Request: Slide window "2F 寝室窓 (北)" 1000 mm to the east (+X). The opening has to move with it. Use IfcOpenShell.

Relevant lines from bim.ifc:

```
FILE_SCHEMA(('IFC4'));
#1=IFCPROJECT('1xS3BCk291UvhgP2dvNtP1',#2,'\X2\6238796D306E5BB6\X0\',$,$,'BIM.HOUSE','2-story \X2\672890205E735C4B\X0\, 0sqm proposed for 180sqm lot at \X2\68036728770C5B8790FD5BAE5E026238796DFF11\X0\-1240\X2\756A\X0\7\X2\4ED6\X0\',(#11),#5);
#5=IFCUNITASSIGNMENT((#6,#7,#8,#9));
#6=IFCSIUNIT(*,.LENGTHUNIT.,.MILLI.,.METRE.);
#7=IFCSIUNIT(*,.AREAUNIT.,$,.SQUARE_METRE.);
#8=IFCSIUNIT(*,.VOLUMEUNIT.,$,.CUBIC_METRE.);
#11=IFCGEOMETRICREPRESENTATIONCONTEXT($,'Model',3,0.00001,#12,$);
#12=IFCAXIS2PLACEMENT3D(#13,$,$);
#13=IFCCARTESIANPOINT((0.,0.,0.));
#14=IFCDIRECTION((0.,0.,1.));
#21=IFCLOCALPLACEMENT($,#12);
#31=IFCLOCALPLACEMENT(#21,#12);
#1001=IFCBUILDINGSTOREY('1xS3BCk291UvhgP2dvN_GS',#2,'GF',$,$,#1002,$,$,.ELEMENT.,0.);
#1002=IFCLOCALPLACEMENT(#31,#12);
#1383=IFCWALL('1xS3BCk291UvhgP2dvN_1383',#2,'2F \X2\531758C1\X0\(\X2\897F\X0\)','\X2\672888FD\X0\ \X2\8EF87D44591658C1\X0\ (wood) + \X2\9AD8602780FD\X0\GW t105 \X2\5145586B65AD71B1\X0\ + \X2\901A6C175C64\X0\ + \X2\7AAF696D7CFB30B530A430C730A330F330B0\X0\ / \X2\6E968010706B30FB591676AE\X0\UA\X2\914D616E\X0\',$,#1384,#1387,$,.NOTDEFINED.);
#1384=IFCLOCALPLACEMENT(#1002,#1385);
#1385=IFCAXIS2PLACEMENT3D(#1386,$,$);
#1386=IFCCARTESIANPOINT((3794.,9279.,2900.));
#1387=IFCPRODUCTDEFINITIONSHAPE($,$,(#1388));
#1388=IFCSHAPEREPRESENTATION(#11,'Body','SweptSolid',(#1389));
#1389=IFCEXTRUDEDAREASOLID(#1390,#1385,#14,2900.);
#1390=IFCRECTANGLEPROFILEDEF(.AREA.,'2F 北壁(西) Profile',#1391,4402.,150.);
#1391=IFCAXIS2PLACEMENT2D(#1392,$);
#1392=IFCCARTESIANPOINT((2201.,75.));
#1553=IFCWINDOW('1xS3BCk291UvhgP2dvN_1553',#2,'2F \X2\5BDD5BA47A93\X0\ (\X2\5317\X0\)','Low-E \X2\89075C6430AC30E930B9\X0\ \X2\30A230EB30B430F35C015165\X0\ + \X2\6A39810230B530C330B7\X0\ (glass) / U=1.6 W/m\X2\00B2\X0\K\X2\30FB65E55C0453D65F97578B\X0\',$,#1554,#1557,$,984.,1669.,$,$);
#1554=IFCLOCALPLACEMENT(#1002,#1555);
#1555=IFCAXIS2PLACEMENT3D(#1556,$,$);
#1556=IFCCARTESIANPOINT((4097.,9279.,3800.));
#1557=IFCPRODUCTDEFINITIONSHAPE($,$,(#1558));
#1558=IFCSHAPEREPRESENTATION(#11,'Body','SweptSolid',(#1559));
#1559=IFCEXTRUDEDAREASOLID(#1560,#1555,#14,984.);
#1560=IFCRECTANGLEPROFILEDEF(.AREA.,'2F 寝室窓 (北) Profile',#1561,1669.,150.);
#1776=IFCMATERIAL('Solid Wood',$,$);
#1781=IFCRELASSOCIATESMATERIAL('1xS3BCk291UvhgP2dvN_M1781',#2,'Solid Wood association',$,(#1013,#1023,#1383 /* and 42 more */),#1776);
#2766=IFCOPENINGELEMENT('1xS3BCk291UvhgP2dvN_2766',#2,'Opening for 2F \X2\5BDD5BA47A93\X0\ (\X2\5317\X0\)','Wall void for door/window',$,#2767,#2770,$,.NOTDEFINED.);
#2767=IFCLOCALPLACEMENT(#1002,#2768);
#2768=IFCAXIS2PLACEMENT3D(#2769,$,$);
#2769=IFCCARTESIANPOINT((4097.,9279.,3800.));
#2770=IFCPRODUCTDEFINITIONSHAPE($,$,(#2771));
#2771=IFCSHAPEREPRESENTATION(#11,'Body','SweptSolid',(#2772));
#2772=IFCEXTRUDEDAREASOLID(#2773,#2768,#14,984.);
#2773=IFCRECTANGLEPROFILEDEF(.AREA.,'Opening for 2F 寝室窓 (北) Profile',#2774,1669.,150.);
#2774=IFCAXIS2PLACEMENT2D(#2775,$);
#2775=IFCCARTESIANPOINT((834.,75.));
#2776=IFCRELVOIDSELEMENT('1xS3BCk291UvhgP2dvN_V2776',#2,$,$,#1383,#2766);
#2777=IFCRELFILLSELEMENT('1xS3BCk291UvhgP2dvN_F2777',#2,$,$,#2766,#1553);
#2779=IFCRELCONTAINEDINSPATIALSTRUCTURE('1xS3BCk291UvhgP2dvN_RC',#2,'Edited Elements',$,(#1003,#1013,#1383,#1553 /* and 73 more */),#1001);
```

```python
import ifcopenshell
import ifcopenshell.api.geometry
import ifcopenshell.util.placement
import ifcopenshell.util.unit

model = ifcopenshell.open("bim.ifc")
unit_scale = ifcopenshell.util.unit.calculate_unit_scale(model)

window = model.by_id(1553)
opening = window.FillsVoids[0].RelatingOpeningElement
wall = opening.VoidsElements[0].RelatingBuildingElement

wall_matrix = ifcopenshell.util.placement.get_local_placement(wall.ObjectPlacement)
shift = wall_matrix[:3, 0] * 1 / unit_scale
before = ifcopenshell.util.placement.get_local_placement(window.ObjectPlacement)[:3, 3].copy()

# The window is not placed relative to its opening, so move both.
for product in (opening, window):
    matrix = ifcopenshell.util.placement.get_local_placement(product.ObjectPlacement)
    matrix[:3, 3] += shift
    ifcopenshell.api.geometry.edit_object_placement(model, product=product, matrix=matrix, is_si=False)

after = ifcopenshell.util.placement.get_local_placement(window.ObjectPlacement)[:3, 3]
print("window moved by", (after - before).round(3) + 0.0)

model.write("bim_v2.ifc")
```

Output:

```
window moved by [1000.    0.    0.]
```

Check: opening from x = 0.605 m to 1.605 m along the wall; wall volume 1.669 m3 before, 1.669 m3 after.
